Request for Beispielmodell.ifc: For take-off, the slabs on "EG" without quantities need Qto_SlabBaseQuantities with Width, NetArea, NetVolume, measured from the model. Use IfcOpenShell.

First a look at what the model holds.

```python
import ifcopenshell
import ifcopenshell.util.element
import ifcopenshell.util.unit

model = ifcopenshell.open("Beispielmodell.ifc")
print(model.schema)
for unit_type in ("LENGTHUNIT", "AREAUNIT", "VOLUMEUNIT"):
    print(unit_type, ifcopenshell.util.unit.calculate_unit_scale(model, unit_type))
storey = next(s for s in model.by_type("IfcBuildingStorey") if s.Name == "EG")
slabs = [e for e in ifcopenshell.util.element.get_decomposition(storey) if e.is_a("IfcSlab")]
for e in sorted(slabs, key=lambda e: e.id()):
    print(e.id(), e.is_a(), e.Name, list(ifcopenshell.util.element.get_psets(e, qtos_only=True)), sep=" | ")
```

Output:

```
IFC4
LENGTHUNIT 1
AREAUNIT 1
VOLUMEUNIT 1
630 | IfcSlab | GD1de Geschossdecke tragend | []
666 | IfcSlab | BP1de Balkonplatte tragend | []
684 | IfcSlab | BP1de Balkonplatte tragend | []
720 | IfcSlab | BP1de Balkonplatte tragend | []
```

```python
import ifcopenshell
import ifcopenshell.api.pset
import ifcopenshell.geom
import ifcopenshell.util.element
import ifcopenshell.util.shape
import ifcopenshell.util.unit

model = ifcopenshell.open("Beispielmodell.ifc")
unit_scale = ifcopenshell.util.unit.calculate_unit_scale(model)
area_scale = ifcopenshell.util.unit.calculate_unit_scale(model, "AREAUNIT")
volume_scale = ifcopenshell.util.unit.calculate_unit_scale(model, "VOLUMEUNIT")
settings = ifcopenshell.geom.settings()

storey = next(s for s in model.by_type("IfcBuildingStorey") if s.Name == "EG")
slabs = [e for e in ifcopenshell.util.element.get_decomposition(storey) if e.is_a("IfcSlab")]

for e in sorted(slabs, key=lambda e: e.id()):
    if ifcopenshell.util.element.get_psets(e, qtos_only=True, should_inherit=False):
        continue
    # Geometry comes back in metres, in the element's own axes.
    shape = ifcopenshell.geom.create_shape(settings, e)
    values = {
        "Width": ifcopenshell.util.shape.get_z(shape.geometry) / unit_scale,
        "NetArea": ifcopenshell.util.shape.get_footprint_area(shape.geometry) / area_scale,
        "NetVolume": ifcopenshell.util.shape.get_volume(shape.geometry) / volume_scale,
    }
    qto = ifcopenshell.api.pset.add_qto(model, product=e, name="Qto_SlabBaseQuantities")
    ifcopenshell.api.pset.edit_qto(model, qto=qto, properties=values)
    print(e.id(), {k: round(v, 3) for k, v in values.items()})

model.write("Beispielmodell_edited.ifc")
```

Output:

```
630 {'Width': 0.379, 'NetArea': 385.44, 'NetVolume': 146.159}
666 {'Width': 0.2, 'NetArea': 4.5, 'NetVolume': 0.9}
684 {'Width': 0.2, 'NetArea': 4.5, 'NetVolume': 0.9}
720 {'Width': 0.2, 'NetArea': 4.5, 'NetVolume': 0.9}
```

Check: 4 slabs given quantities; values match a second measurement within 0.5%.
